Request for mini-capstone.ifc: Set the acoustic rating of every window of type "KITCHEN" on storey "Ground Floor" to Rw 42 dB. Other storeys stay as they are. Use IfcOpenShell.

First a look at what the model holds.

```python
import ifcopenshell
import ifcopenshell.util.element

model = ifcopenshell.open("mini-capstone.ifc")
print(model.schema)
storey = next(s for s in model.by_type("IfcBuildingStorey") if s.Name == "Ground Floor")
windows = [e for e in ifcopenshell.util.element.get_decomposition(storey) if e.is_a("IfcWindow")]
seen = {}
for e in windows:
    element_type = ifcopenshell.util.element.get_type(e)
    key = (element_type.Name if element_type != e and element_type else None, ifcopenshell.util.element.get_pset(e, "Pset_WindowCommon", "AcousticRating"))
    seen[key] = seen.get(key, 0) + 1
for (name, value), count in sorted(seen.items(), key=str):
    print(count, "x", name, "|", value)
```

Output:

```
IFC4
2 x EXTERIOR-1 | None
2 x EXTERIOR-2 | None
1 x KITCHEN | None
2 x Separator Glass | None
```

```python
import ifcopenshell
import ifcopenshell.api.pset
import ifcopenshell.util.element

model = ifcopenshell.open("mini-capstone.ifc")

storey = next(s for s in model.by_type("IfcBuildingStorey") if s.Name == "Ground Floor")
windows = [e for e in ifcopenshell.util.element.get_decomposition(storey) if e.is_a("IfcWindow")]

count = 0
for e in windows:
    element_type = ifcopenshell.util.element.get_type(e)
    if element_type in (None, e) or element_type.Name != "KITCHEN":
        continue
    # add_pset returns the element's existing set when there is one.
    pset = ifcopenshell.api.pset.add_pset(model, product=e, name="Pset_WindowCommon")
    ifcopenshell.api.pset.edit_pset(model, pset=pset, properties={"AcousticRating": "Rw 42 dB"})
    count += 1

print(count, "windows updated")

model.write("mini-capstone_v2.ifc")
```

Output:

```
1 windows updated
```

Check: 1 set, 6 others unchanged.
